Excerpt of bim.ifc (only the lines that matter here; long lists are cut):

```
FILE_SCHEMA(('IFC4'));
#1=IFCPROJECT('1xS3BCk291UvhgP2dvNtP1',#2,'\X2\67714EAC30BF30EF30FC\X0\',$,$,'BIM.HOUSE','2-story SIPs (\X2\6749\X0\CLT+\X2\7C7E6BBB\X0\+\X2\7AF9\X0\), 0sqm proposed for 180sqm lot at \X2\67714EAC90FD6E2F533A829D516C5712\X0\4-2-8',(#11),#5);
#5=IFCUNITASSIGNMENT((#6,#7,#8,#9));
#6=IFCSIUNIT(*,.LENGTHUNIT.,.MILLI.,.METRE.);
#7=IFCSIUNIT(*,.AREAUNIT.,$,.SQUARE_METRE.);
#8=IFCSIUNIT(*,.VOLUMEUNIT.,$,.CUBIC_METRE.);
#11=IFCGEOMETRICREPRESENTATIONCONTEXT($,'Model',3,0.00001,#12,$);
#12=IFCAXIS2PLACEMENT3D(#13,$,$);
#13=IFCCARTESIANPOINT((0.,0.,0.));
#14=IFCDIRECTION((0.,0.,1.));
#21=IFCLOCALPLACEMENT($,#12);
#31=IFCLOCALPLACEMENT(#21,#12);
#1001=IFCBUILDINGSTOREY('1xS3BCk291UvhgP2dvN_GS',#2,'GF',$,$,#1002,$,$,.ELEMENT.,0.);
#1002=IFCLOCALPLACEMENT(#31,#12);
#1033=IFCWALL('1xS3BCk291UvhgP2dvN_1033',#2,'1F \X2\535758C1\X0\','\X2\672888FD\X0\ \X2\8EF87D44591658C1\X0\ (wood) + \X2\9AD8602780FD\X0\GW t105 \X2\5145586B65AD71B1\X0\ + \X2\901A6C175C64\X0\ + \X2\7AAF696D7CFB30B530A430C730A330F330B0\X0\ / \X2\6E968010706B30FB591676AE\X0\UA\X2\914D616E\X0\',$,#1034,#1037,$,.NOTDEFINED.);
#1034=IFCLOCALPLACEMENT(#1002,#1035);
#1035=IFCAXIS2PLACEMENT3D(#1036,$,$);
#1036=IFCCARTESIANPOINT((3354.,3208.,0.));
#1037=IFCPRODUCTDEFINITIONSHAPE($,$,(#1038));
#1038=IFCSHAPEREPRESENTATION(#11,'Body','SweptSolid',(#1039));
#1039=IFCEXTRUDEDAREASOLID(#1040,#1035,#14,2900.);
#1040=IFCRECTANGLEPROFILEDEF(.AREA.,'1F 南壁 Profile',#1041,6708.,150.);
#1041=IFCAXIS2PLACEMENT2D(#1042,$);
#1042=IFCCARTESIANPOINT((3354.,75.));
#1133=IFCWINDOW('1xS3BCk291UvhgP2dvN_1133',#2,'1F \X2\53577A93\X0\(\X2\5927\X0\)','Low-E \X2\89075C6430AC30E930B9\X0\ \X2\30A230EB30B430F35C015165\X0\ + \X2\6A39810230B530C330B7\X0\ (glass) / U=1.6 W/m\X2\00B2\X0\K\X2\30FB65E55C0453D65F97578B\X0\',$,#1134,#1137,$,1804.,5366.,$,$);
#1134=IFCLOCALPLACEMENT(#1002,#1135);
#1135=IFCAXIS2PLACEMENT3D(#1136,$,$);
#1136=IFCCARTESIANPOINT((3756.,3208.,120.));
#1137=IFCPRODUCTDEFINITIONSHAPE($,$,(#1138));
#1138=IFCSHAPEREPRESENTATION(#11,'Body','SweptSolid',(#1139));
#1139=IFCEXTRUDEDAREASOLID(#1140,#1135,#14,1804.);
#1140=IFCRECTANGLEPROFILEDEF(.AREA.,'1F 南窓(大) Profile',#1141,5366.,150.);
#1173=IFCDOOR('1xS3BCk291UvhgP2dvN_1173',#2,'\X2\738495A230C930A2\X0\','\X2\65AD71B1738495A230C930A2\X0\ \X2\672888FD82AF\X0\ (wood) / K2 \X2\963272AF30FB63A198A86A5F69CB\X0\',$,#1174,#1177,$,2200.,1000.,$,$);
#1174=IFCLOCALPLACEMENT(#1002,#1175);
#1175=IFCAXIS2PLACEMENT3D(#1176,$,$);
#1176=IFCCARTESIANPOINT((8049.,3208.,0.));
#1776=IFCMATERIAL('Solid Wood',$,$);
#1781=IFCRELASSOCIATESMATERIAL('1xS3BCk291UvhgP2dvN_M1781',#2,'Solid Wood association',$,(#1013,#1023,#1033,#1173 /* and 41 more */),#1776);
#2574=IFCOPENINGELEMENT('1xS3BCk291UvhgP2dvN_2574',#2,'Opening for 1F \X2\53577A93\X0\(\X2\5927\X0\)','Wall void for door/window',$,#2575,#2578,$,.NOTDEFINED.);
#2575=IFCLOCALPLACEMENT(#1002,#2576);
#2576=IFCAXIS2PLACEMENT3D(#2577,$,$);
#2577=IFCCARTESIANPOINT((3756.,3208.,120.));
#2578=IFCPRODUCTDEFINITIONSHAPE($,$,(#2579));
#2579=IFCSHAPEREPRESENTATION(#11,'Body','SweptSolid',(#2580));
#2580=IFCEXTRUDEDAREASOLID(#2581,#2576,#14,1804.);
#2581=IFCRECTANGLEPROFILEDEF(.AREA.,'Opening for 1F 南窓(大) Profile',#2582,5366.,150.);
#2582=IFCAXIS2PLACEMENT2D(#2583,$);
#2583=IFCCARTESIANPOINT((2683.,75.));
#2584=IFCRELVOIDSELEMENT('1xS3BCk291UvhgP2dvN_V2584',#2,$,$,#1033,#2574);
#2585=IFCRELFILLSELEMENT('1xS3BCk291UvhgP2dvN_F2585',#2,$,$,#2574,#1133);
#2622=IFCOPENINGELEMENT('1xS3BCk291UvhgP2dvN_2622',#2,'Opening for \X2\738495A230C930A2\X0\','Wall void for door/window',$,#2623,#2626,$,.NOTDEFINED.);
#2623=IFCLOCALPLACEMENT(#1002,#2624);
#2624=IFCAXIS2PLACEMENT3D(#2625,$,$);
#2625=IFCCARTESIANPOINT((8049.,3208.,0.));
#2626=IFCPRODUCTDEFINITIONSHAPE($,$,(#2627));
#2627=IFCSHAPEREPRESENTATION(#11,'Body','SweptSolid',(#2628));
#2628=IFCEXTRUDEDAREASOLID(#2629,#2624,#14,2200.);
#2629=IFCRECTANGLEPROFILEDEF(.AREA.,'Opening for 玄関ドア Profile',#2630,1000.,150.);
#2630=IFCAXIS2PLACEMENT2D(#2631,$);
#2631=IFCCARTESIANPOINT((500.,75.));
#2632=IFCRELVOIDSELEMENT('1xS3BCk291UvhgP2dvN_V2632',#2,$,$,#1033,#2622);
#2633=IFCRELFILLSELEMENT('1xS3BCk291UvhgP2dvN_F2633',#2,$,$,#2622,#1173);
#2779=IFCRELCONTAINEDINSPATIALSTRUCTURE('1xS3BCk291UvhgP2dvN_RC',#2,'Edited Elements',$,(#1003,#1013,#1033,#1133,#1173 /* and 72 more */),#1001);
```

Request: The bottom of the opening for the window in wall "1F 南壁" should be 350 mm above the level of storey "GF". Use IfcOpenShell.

```python
import numpy as np
import ifcopenshell
import ifcopenshell.api.geometry
import ifcopenshell.geom
import ifcopenshell.util.element
import ifcopenshell.util.placement
import ifcopenshell.util.shape
import ifcopenshell.util.unit

model = ifcopenshell.open("bim.ifc")
unit_scale = ifcopenshell.util.unit.calculate_unit_scale(model)

window = model.by_guid("1xS3BCk291UvhgP2dvN_1133")
opening = window.FillsVoids[0].RelatingOpeningElement
storey = ifcopenshell.util.element.get_container(window, ifc_class="IfcBuildingStorey")
level = ifcopenshell.util.placement.get_local_placement(storey.ObjectPlacement)[2, 3]

# The opening's origin need not be at the sill, so measure its lowest point.
shape = ifcopenshell.geom.create_shape(ifcopenshell.geom.settings(), opening)
bottom = ifcopenshell.util.shape.get_shape_bottom_elevation(shape, shape.geometry) / unit_scale
dz = level + 0.35 / unit_scale - bottom

shift = np.array([0.0, 0.0, dz])
# The window is not placed relative to its opening, so move both.
for product in (opening, window):
    matrix = ifcopenshell.util.placement.get_local_placement(product.ObjectPlacement)
    matrix[:3, 3] += shift
    ifcopenshell.api.geometry.edit_object_placement(model, product=product, matrix=matrix, is_si=False)

print(f"moved by {dz * unit_scale:+.3f} m")

model.write("bim_v2.ifc")
```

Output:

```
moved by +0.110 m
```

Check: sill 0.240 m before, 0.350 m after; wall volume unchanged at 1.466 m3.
